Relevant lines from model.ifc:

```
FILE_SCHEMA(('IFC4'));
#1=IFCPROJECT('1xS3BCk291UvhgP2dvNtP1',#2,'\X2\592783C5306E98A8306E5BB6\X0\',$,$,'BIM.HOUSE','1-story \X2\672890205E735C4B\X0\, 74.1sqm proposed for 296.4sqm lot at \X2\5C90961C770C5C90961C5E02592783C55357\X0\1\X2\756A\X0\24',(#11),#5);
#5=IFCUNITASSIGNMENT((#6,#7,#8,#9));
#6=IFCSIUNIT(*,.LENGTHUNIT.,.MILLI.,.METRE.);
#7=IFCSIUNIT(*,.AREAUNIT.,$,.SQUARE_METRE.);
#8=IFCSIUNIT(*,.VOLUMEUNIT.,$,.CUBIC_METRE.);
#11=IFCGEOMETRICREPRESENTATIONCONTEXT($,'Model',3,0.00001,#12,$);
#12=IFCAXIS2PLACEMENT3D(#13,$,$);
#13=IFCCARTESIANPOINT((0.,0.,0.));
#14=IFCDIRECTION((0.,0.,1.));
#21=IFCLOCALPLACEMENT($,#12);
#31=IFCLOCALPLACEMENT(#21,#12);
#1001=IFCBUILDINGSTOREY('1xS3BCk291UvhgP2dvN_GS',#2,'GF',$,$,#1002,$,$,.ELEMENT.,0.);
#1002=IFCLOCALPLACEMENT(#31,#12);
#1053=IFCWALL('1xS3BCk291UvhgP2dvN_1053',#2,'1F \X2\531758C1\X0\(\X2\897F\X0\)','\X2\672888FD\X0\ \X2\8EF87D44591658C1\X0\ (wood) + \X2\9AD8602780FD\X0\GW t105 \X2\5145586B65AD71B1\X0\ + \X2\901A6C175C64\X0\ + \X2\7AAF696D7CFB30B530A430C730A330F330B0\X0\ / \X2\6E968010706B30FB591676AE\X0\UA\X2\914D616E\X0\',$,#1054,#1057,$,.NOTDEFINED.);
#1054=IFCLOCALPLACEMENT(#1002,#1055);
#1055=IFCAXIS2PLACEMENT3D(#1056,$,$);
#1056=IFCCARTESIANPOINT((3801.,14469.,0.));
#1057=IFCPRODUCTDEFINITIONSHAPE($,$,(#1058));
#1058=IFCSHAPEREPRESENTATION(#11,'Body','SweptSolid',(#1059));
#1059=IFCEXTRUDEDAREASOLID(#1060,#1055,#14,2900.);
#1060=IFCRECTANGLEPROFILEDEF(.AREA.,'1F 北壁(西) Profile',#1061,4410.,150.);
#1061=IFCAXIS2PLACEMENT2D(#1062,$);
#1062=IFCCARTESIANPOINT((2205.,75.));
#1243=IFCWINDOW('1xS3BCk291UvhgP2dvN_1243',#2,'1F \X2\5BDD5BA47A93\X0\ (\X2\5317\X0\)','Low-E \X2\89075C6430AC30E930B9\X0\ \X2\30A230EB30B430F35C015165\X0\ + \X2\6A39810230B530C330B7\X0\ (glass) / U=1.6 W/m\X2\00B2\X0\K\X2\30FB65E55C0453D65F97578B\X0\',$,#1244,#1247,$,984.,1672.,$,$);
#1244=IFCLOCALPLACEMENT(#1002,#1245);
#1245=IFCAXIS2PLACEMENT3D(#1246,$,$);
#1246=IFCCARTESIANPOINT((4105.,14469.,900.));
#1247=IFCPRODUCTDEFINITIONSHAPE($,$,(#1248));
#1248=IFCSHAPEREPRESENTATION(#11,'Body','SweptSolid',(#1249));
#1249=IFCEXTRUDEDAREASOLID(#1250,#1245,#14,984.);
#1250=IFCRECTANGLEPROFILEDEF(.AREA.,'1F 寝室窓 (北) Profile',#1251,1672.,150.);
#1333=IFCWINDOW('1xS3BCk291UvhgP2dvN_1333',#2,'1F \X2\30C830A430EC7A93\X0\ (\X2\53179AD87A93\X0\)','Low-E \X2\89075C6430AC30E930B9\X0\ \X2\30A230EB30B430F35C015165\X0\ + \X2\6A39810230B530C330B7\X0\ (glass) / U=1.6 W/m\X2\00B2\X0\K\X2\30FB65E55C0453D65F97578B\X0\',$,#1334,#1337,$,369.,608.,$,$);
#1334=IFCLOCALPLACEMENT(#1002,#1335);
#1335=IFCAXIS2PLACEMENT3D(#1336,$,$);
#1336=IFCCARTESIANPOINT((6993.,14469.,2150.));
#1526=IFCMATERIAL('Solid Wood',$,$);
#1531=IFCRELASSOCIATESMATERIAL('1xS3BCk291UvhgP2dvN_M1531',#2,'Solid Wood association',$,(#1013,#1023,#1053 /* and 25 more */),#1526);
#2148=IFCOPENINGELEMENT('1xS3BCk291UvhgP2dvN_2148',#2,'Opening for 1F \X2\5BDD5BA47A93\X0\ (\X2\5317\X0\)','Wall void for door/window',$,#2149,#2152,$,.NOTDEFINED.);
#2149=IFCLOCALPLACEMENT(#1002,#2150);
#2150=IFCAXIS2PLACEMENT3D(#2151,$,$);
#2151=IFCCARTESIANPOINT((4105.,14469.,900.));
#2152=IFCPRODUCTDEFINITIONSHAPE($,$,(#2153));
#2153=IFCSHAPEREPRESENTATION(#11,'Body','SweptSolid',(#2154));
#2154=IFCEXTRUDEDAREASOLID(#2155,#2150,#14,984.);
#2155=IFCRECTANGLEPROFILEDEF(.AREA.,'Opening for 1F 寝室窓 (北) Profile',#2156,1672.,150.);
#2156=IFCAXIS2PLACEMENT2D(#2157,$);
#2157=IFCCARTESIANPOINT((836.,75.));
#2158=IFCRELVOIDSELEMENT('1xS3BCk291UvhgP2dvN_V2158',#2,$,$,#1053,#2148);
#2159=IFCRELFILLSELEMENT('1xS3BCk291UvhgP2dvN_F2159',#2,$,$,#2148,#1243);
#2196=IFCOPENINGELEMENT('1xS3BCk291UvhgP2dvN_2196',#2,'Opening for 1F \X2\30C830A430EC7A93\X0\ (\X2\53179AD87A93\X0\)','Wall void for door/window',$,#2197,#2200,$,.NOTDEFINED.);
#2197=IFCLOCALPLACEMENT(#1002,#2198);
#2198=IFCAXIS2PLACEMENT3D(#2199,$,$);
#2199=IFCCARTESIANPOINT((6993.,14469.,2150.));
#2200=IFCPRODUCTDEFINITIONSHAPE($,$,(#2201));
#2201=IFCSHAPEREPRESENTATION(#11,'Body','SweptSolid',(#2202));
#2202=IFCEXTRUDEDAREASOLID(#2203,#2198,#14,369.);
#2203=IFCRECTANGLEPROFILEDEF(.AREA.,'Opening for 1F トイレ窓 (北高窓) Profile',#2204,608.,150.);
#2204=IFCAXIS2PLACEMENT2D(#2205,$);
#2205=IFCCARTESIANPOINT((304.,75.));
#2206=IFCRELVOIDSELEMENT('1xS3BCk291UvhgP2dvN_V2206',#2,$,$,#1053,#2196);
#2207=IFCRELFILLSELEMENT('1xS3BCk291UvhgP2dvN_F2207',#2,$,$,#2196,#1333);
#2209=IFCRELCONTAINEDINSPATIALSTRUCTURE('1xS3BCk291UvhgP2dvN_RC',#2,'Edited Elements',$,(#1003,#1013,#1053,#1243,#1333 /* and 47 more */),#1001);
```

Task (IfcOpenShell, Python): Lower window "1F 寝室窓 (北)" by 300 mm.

```python
import numpy as np
import ifcopenshell
import ifcopenshell.api.geometry
import ifcopenshell.util.placement
import ifcopenshell.util.unit

model = ifcopenshell.open("model.ifc")
unit_scale = ifcopenshell.util.unit.calculate_unit_scale(model)

window = model.by_id(1243)
opening = window.FillsVoids[0].RelatingOpeningElement
dz = -0.3 / unit_scale

shift = np.array([0.0, 0.0, dz])
# The window is not placed relative to its opening, so move both.
for product in (opening, window):
    matrix = ifcopenshell.util.placement.get_local_placement(product.ObjectPlacement)
    matrix[:3, 3] += shift
    ifcopenshell.api.geometry.edit_object_placement(model, product=product, matrix=matrix, is_si=False)

print(f"moved by {dz * unit_scale:+.3f} m")

model.write("model_edited.ifc")
```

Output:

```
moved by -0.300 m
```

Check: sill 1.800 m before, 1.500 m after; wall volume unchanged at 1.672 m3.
